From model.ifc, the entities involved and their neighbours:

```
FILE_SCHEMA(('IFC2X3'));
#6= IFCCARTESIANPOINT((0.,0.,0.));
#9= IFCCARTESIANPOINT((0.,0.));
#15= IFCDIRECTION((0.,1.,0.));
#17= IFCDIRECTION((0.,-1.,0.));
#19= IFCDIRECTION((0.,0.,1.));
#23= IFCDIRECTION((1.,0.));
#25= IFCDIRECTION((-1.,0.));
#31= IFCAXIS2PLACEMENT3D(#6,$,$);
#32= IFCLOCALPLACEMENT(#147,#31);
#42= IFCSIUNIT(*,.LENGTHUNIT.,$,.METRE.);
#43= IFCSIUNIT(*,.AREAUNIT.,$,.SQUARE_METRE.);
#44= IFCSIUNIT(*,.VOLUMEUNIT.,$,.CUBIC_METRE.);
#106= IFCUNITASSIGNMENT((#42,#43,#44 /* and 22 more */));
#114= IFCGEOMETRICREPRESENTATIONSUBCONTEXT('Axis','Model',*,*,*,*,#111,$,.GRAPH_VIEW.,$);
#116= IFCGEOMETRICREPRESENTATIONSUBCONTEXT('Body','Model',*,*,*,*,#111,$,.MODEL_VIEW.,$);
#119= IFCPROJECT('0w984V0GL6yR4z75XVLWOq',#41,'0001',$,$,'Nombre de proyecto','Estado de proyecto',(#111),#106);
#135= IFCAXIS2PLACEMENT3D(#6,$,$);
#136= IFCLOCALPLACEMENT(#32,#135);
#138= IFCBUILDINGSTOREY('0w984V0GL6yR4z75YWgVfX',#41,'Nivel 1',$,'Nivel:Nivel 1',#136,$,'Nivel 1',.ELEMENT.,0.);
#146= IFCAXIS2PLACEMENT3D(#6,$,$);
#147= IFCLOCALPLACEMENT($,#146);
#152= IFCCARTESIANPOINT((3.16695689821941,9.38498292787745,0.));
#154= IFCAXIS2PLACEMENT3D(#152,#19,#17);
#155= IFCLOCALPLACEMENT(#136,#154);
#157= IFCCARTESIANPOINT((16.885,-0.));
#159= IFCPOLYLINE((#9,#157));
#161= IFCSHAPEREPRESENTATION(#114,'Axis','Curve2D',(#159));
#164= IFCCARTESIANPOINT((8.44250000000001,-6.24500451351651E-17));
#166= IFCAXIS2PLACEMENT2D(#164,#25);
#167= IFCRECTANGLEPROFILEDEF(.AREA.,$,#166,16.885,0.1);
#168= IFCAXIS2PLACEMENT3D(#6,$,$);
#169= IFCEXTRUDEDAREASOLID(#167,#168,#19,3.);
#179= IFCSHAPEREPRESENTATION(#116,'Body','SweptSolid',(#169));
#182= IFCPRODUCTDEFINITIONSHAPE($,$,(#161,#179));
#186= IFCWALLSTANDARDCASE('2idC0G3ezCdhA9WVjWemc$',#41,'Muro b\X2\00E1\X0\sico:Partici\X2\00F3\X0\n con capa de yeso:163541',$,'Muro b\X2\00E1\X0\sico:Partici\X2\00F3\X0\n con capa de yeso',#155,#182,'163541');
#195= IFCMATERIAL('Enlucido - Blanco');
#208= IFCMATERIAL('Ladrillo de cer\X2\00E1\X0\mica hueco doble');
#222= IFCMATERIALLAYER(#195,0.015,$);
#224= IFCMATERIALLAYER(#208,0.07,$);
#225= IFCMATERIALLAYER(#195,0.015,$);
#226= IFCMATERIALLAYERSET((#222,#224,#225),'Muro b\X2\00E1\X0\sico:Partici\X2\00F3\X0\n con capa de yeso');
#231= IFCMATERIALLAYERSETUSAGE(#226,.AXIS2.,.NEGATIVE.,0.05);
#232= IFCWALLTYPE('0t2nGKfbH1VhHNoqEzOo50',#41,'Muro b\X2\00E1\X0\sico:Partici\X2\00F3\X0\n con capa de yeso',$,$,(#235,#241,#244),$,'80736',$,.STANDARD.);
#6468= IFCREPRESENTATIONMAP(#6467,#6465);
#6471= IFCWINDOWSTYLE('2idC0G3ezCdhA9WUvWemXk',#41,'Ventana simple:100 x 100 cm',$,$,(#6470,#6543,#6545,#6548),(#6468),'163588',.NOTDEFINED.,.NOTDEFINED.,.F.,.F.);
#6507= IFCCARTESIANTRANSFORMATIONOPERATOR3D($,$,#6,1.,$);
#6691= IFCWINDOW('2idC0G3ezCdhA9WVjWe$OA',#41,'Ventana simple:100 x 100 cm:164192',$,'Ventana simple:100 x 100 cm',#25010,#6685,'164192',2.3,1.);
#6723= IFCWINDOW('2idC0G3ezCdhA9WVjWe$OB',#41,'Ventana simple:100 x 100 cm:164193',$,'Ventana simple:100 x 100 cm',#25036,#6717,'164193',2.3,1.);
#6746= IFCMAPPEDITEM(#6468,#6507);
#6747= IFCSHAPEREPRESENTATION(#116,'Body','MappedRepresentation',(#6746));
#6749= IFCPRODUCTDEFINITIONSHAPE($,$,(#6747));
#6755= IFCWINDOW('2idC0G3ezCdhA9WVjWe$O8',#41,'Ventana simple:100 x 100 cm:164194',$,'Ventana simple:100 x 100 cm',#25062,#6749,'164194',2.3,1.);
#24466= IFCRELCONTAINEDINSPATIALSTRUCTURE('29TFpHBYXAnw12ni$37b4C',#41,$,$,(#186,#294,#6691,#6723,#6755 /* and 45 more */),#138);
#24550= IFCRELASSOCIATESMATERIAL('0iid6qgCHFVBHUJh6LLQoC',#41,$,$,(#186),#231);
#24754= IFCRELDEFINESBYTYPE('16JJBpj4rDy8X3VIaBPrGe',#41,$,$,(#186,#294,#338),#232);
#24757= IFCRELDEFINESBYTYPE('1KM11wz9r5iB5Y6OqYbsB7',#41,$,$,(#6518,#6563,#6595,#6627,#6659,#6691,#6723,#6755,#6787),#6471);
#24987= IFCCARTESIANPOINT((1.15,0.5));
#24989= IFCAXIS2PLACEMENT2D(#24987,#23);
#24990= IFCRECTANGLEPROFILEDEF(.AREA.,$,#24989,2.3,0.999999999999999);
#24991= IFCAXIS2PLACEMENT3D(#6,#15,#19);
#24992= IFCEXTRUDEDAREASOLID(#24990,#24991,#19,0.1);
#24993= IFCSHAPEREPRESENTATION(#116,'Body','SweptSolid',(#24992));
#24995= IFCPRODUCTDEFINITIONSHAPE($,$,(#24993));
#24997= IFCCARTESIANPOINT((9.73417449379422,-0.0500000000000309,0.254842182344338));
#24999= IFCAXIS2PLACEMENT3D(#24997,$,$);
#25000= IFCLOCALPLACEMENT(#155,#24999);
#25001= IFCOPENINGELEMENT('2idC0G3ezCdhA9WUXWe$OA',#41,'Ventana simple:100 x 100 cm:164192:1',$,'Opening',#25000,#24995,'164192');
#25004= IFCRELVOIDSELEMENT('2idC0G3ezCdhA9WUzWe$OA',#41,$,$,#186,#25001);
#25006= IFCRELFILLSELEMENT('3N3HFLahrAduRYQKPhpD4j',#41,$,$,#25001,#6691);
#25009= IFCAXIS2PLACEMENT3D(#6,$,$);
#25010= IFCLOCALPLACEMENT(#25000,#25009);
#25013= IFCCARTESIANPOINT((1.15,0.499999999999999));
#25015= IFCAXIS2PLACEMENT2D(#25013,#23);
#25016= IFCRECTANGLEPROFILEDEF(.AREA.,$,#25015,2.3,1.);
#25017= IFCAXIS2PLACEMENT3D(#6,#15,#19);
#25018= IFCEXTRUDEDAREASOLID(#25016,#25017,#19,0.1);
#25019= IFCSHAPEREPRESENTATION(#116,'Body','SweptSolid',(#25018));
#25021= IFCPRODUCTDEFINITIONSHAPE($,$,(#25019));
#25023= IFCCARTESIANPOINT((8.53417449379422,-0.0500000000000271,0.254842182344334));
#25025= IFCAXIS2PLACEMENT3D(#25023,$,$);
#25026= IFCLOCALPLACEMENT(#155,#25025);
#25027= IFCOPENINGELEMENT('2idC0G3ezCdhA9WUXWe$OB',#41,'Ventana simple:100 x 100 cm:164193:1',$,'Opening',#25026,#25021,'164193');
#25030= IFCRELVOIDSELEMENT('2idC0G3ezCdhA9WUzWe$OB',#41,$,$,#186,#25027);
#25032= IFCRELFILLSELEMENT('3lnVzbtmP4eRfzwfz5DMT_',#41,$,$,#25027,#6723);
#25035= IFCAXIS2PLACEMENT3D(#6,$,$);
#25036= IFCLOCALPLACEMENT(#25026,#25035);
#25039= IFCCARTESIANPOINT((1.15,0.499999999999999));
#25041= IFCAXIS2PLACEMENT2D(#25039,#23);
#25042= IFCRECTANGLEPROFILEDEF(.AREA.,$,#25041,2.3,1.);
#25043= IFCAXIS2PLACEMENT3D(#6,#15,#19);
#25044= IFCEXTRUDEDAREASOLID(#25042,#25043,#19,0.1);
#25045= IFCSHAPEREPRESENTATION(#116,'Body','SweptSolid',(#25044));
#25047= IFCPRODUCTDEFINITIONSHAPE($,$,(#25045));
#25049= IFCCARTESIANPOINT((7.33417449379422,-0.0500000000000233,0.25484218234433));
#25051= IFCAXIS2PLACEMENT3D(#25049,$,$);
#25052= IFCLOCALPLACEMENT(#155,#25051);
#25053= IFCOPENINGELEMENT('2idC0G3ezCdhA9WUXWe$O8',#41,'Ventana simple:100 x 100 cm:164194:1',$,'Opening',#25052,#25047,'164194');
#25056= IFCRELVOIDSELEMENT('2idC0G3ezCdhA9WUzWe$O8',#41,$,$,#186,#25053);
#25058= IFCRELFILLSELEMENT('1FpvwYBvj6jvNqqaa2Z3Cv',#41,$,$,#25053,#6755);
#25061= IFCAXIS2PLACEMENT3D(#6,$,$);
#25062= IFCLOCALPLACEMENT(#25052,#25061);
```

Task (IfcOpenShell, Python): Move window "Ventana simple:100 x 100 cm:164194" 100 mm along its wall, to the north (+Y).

```python
import ifcopenshell
import ifcopenshell.api.geometry
import ifcopenshell.util.placement
import ifcopenshell.util.unit

model = ifcopenshell.open("model.ifc")
unit_scale = ifcopenshell.util.unit.calculate_unit_scale(model)

window = model.by_id(6755)
opening = window.FillsVoids[0].RelatingOpeningElement
wall = opening.VoidsElements[0].RelatingBuildingElement

wall_matrix = ifcopenshell.util.placement.get_local_placement(wall.ObjectPlacement)
shift = wall_matrix[:3, 0] * -0.1 / unit_scale
before = ifcopenshell.util.placement.get_local_placement(window.ObjectPlacement)[:3, 3].copy()

# The window is placed relative to its opening, so it follows when the opening moves.
matrix = ifcopenshell.util.placement.get_local_placement(opening.ObjectPlacement)
matrix[:3, 3] += shift
ifcopenshell.api.geometry.edit_object_placement(
    model, product=opening, matrix=matrix, is_si=False, should_transform_children=True
)

after = ifcopenshell.util.placement.get_local_placement(window.ObjectPlacement)[:3, 3]
print("window moved by", (after - before).round(3) + 0.0)

model.write("model_updated.ifc")
```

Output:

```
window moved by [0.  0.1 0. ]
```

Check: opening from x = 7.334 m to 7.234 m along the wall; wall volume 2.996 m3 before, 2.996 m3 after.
